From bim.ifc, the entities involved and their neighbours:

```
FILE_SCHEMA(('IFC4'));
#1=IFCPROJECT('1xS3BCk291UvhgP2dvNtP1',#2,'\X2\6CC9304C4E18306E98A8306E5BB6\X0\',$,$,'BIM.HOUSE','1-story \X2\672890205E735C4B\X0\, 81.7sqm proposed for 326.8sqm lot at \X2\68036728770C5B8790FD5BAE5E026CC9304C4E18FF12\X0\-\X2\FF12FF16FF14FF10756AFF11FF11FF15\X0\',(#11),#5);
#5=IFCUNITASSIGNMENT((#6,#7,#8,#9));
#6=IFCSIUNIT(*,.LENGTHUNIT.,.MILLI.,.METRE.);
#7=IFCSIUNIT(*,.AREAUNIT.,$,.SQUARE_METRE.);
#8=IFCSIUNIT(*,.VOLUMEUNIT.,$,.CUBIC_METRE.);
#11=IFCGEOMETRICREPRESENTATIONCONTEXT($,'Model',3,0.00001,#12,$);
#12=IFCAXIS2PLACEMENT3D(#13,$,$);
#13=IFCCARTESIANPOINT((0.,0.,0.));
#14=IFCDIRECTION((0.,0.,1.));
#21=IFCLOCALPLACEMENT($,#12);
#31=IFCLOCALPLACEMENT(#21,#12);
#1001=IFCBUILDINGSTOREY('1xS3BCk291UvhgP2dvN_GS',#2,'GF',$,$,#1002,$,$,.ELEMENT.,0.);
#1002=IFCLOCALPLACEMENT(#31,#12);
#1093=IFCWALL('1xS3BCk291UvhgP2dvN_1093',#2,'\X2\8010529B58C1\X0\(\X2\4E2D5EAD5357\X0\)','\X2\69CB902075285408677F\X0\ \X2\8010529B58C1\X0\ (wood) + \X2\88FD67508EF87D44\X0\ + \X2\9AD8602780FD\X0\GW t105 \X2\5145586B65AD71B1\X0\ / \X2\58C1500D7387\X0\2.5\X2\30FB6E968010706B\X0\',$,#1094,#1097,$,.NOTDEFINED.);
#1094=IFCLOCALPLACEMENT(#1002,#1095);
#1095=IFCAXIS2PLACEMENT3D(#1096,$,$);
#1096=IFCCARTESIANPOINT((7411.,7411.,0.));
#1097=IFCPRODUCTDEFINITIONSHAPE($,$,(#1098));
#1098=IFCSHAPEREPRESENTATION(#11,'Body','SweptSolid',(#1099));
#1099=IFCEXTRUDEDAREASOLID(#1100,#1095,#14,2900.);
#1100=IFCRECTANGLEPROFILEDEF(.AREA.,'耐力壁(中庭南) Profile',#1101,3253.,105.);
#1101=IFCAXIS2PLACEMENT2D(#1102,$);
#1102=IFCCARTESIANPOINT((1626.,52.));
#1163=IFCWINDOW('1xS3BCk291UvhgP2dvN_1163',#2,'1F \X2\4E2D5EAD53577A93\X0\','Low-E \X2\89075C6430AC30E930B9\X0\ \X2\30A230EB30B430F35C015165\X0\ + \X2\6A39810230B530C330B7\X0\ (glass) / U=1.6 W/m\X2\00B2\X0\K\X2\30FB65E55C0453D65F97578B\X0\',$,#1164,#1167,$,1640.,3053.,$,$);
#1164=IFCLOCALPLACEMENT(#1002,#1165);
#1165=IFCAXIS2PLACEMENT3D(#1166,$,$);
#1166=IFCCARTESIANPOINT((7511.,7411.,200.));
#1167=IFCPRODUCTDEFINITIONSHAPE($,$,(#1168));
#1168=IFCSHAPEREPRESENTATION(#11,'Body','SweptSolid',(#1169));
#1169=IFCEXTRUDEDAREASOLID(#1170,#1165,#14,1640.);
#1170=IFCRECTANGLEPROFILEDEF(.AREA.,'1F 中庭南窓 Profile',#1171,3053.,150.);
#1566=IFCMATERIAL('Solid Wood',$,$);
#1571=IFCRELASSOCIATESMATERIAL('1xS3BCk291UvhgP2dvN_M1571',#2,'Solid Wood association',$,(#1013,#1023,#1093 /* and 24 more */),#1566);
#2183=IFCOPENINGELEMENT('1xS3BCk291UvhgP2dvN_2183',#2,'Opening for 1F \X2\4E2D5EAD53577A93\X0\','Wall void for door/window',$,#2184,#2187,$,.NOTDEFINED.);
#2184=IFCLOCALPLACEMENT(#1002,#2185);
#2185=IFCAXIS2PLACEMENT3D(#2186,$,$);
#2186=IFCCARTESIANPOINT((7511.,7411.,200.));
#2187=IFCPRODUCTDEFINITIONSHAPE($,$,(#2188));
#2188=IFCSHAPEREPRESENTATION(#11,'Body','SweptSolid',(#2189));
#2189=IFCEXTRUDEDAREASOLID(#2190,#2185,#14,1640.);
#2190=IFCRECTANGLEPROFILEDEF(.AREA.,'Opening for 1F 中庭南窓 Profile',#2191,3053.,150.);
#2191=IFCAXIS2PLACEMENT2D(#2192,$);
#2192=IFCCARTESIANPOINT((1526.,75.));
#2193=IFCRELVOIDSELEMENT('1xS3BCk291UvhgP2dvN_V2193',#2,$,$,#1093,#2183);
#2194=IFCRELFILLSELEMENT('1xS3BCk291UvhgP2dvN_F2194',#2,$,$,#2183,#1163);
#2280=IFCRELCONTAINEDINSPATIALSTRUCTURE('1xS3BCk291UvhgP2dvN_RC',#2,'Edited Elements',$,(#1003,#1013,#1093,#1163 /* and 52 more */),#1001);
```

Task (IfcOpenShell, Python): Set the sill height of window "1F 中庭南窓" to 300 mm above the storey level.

```python
import numpy as np
import ifcopenshell
import ifcopenshell.api.geometry
import ifcopenshell.geom
import ifcopenshell.util.element
import ifcopenshell.util.placement
import ifcopenshell.util.shape
import ifcopenshell.util.unit

model = ifcopenshell.open("bim.ifc")
unit_scale = ifcopenshell.util.unit.calculate_unit_scale(model)

window = model.by_id(1163)
opening = window.FillsVoids[0].RelatingOpeningElement
storey = ifcopenshell.util.element.get_container(window, ifc_class="IfcBuildingStorey")
level = ifcopenshell.util.placement.get_local_placement(storey.ObjectPlacement)[2, 3]

# The opening's origin need not be at the sill, so measure its lowest point.
shape = ifcopenshell.geom.create_shape(ifcopenshell.geom.settings(), opening)
bottom = ifcopenshell.util.shape.get_shape_bottom_elevation(shape, shape.geometry) / unit_scale
dz = level + 0.3 / unit_scale - bottom

shift = np.array([0.0, 0.0, dz])
# The window is not placed relative to its opening, so move both.
for product in (opening, window):
    matrix = ifcopenshell.util.placement.get_local_placement(product.ObjectPlacement)
    matrix[:3, 3] += shift
    ifcopenshell.api.geometry.edit_object_placement(model, product=product, matrix=matrix, is_si=False)

print(f"moved by {dz * unit_scale:+.3f} m")

model.write("bim_edited.ifc")
```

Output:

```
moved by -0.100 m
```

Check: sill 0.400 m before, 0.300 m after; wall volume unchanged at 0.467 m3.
